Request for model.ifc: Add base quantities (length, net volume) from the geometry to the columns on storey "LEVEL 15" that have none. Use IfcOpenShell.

First a look at what the model holds.

```python
import ifcopenshell
import ifcopenshell.util.element
import ifcopenshell.util.unit

model = ifcopenshell.open("model.ifc")
print(model.schema)
for unit_type in ("LENGTHUNIT", "AREAUNIT", "VOLUMEUNIT"):
    print(unit_type, ifcopenshell.util.unit.calculate_unit_scale(model, unit_type))
storey = next(s for s in model.by_type("IfcBuildingStorey") if s.Name == "LEVEL 15")
columns = [e for e in ifcopenshell.util.element.get_decomposition(storey) if e.is_a("IfcColumn")]
for e in sorted(columns, key=lambda e: e.id()):
    print(e.id(), e.is_a(), e.Name, list(ifcopenshell.util.element.get_psets(e, qtos_only=True)), sep=" | ")
```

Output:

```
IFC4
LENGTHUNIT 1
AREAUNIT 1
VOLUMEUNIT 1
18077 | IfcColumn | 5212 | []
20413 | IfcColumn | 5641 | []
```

```python
import ifcopenshell
import ifcopenshell.api.pset
import ifcopenshell.geom
import ifcopenshell.util.element
import ifcopenshell.util.shape
import ifcopenshell.util.unit

model = ifcopenshell.open("model.ifc")
unit_scale = ifcopenshell.util.unit.calculate_unit_scale(model)
volume_scale = ifcopenshell.util.unit.calculate_unit_scale(model, "VOLUMEUNIT")
settings = ifcopenshell.geom.settings()

storey = next(s for s in model.by_type("IfcBuildingStorey") if s.Name == "LEVEL 15")
columns = [e for e in ifcopenshell.util.element.get_decomposition(storey) if e.is_a("IfcColumn")]

for e in sorted(columns, key=lambda e: e.id()):
    if ifcopenshell.util.element.get_psets(e, qtos_only=True, should_inherit=False):
        continue
    # Geometry comes back in metres, in the element's own axes.
    shape = ifcopenshell.geom.create_shape(settings, e)
    values = {
        "Length": ifcopenshell.util.shape.get_z(shape.geometry) / unit_scale,
        "NetVolume": ifcopenshell.util.shape.get_volume(shape.geometry) / volume_scale,
    }
    qto = ifcopenshell.api.pset.add_qto(model, product=e, name="Qto_ColumnBaseQuantities")
    ifcopenshell.api.pset.edit_qto(model, qto=qto, properties=values)
    print(e.id(), {k: round(v, 3) for k, v in values.items()})

model.write("model_v2.ifc")
```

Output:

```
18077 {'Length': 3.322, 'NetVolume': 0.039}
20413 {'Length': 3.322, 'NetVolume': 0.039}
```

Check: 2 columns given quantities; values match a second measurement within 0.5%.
